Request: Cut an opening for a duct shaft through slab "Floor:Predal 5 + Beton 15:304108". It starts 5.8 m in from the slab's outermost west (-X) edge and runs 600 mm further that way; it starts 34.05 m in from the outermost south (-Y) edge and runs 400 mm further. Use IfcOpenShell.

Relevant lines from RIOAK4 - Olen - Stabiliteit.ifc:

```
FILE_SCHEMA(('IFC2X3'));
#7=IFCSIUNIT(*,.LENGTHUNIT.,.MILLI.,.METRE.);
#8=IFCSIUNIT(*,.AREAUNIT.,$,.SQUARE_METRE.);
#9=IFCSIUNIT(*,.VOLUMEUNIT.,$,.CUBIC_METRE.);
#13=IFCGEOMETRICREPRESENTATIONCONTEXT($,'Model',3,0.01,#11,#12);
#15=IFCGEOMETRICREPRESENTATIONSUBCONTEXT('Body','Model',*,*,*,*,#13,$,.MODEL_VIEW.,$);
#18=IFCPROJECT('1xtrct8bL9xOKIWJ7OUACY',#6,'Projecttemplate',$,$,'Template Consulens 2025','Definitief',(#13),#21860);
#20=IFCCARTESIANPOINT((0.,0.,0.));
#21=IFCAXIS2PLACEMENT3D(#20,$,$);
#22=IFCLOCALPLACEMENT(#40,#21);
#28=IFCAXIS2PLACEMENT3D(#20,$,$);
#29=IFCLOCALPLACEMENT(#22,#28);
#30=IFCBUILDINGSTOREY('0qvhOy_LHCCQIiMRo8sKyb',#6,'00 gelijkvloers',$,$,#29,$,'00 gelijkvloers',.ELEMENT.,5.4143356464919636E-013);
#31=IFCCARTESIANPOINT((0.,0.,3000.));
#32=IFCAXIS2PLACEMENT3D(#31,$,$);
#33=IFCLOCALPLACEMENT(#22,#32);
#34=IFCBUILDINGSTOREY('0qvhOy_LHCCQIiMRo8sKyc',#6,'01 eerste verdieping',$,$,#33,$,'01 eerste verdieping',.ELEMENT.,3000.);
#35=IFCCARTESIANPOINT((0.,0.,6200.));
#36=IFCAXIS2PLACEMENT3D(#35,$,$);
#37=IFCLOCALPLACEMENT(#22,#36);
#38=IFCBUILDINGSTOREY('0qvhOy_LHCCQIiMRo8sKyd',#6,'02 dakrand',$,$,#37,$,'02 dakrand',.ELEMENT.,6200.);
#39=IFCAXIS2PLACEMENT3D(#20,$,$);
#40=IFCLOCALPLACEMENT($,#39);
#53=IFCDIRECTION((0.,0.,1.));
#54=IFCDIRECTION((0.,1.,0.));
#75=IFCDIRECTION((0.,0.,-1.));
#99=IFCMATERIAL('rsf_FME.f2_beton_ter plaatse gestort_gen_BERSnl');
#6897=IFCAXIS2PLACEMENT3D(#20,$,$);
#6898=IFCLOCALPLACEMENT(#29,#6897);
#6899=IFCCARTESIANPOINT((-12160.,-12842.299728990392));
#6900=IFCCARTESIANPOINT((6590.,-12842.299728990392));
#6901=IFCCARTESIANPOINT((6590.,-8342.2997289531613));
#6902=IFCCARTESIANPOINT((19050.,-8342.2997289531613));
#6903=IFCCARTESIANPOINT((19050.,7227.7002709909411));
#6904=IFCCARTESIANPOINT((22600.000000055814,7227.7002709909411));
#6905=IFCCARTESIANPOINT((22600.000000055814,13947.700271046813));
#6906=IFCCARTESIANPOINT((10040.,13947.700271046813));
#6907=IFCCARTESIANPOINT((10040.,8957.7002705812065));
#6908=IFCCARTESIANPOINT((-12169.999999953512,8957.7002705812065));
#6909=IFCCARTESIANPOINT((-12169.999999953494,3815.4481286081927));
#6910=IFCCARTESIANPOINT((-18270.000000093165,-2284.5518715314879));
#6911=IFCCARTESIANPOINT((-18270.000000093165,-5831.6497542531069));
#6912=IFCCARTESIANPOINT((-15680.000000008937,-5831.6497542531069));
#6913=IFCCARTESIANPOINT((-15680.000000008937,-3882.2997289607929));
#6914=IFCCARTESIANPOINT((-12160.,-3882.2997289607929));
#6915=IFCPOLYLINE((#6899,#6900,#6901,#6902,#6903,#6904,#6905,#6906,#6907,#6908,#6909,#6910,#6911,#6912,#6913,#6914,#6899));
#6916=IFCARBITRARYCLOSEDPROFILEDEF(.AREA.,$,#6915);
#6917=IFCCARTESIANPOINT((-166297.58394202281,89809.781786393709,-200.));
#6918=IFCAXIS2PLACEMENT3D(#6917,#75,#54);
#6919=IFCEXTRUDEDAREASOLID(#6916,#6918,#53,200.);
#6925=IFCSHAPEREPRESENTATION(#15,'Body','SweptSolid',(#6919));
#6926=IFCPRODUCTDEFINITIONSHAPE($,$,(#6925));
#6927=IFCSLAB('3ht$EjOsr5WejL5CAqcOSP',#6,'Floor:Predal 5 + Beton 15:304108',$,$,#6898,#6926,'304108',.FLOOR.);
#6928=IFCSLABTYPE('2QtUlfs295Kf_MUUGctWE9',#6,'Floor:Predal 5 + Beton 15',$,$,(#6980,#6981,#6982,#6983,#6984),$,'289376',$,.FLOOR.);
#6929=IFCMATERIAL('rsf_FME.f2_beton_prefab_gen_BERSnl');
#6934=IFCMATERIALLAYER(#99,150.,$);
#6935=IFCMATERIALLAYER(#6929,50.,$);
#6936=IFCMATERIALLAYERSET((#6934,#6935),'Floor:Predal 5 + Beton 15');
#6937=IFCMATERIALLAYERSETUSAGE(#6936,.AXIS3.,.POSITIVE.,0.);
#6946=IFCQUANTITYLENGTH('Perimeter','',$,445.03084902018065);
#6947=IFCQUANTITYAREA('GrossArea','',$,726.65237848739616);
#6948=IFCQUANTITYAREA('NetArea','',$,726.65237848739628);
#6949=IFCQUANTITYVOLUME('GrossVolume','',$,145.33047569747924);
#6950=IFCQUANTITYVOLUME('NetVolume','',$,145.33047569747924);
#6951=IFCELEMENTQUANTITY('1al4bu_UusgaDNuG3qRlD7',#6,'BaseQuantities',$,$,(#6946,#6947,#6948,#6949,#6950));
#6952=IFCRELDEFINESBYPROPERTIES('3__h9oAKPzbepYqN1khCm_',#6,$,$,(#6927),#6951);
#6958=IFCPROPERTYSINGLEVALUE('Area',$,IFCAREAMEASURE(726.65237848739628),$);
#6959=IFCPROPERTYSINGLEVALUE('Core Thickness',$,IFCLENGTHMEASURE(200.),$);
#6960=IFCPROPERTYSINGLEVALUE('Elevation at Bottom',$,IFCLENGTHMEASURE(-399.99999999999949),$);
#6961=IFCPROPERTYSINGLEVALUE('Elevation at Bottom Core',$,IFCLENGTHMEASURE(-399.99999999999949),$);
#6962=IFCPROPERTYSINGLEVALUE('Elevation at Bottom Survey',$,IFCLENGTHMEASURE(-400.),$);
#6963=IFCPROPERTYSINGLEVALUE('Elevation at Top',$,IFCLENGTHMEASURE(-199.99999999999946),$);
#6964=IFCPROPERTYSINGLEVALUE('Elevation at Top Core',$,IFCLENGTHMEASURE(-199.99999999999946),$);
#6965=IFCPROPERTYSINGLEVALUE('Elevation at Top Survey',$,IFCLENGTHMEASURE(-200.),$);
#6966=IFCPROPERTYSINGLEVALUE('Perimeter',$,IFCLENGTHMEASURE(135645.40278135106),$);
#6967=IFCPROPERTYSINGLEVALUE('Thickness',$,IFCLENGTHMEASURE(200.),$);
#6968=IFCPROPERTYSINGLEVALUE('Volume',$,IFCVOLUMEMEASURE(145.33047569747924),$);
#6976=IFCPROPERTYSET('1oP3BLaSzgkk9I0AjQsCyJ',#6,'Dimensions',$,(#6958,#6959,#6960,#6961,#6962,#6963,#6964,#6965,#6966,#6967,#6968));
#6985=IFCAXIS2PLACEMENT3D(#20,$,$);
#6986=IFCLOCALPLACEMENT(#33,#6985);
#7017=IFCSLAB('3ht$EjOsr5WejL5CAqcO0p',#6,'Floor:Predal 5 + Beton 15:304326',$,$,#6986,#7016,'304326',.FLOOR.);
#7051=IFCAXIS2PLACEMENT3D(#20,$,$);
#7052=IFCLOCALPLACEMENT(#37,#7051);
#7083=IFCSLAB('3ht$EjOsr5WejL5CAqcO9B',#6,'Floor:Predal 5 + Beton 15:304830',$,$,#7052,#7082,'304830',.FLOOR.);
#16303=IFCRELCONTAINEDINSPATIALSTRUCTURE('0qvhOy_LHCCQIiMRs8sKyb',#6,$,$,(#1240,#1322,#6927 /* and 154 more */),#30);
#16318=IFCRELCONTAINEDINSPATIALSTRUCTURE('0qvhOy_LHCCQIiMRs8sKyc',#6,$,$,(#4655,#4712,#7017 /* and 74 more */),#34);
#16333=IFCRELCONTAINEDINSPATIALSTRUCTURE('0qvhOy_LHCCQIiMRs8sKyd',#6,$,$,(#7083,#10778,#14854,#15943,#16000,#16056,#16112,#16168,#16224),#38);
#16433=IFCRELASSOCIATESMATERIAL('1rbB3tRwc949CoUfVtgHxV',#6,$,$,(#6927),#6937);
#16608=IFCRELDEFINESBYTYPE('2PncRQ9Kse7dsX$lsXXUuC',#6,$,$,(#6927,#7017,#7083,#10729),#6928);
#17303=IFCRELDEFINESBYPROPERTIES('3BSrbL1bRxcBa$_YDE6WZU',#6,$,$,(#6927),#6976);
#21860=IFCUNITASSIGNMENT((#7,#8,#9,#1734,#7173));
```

```python
import numpy as np
import ifcopenshell
import ifcopenshell.api.feature
import ifcopenshell.api.geometry
import ifcopenshell.api.pset
import ifcopenshell.api.root
import ifcopenshell.geom
import ifcopenshell.util.element
import ifcopenshell.util.placement
import ifcopenshell.util.representation
import ifcopenshell.util.shape
import ifcopenshell.util.unit

model = ifcopenshell.open("RIOAK4 - Olen - Stabiliteit.ifc")
unit_scale = ifcopenshell.util.unit.calculate_unit_scale(model)
area_scale = ifcopenshell.util.unit.calculate_unit_scale(model, "AREAUNIT")
volume_scale = ifcopenshell.util.unit.calculate_unit_scale(model, "VOLUMEUNIT")
settings = ifcopenshell.geom.settings()


def volume(element):
    """Net volume in cubic metres, openings subtracted."""
    shape = ifcopenshell.geom.create_shape(settings, element)
    return ifcopenshell.util.shape.get_volume(shape.geometry)


slab = model.by_guid("3ht$EjOsr5WejL5CAqcOSP")
before = volume(slab)

# Extent in the slab's own axes, in metres. The edges named are its -X and -Y sides.
slab_shape = ifcopenshell.geom.create_shape(settings, slab)
vertices = ifcopenshell.util.shape.get_vertices(slab_shape.geometry)
x_min, y_min, bottom = vertices.min(axis=0)
top = vertices[:, 2].max()

opening = ifcopenshell.api.root.create_entity(model, ifc_class="IfcOpeningElement", name="Duct shaft opening")
context = ifcopenshell.util.representation.get_context(model, "Model", "Body", "MODEL_VIEW")
width, depth = 0.6, 0.4
outline = [(0.0, 0.0), (width, 0.0), (width, depth), (0.0, depth), (0.0, 0.0)]
# Overshoot both faces by 50 mm so the cut is clean.
shape = ifcopenshell.api.geometry.add_slab_representation(
    model, context=context, depth=top - bottom + 0.1, polyline=outline
)
ifcopenshell.api.geometry.assign_representation(model, product=opening, representation=shape)

matrix = ifcopenshell.util.placement.get_local_placement(slab.ObjectPlacement)
matrix[:, 3] = matrix @ np.append(np.array([x_min + 5.8, y_min + 34.05, bottom - 0.05]) / unit_scale, 1.0)
ifcopenshell.api.geometry.edit_object_placement(model, product=opening, matrix=matrix, is_si=False)
ifcopenshell.api.feature.add_feature(model, feature=opening, element=slab)

after = volume(slab)

# Update the slab's stored quantities.
qto = model.by_id(ifcopenshell.util.element.get_pset(slab, "BaseQuantities", should_inherit=False)["id"])
ifcopenshell.api.pset.edit_qto(model, qto=qto, properties={
    "NetArea": after / (top - bottom) / area_scale,
    "NetVolume": after / volume_scale,
})
pset = model.by_id(ifcopenshell.util.element.get_pset(slab, "Dimensions", should_inherit=False)["id"])
ifcopenshell.api.pset.edit_pset(model, pset=pset, properties={
    "Area": model.create_entity("IfcAreaMeasure", after / (top - bottom) / area_scale),
    "Volume": model.create_entity("IfcVolumeMeasure", after / volume_scale),
})

print(f"slab volume {before:.3f} -> {after:.3f} m3")

model.write("RIOAK4 - Olen - Stabiliteit_rev.ifc")
```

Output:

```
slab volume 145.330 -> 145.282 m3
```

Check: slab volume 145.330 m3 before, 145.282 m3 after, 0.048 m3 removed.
